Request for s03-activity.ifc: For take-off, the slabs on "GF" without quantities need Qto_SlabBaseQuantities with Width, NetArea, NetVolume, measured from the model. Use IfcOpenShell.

First a look at what the model holds.

```python
import ifcopenshell
import ifcopenshell.util.element
import ifcopenshell.util.unit

model = ifcopenshell.open("s03-activity.ifc")
print(model.schema)
for unit_type in ("LENGTHUNIT", "AREAUNIT", "VOLUMEUNIT"):
    print(unit_type, ifcopenshell.util.unit.calculate_unit_scale(model, unit_type))
storey = next(s for s in model.by_type("IfcBuildingStorey") if s.Name == "GF")
slabs = [e for e in ifcopenshell.util.element.get_decomposition(storey) if e.is_a("IfcSlab")]
for e in sorted(slabs, key=lambda e: e.id()):
    print(e.id(), e.is_a(), e.Name, list(ifcopenshell.util.element.get_psets(e, qtos_only=True)), sep=" | ")
```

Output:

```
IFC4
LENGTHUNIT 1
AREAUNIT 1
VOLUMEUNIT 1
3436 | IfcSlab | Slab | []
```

```python
import ifcopenshell
import ifcopenshell.api.pset
import ifcopenshell.geom
import ifcopenshell.util.element
import ifcopenshell.util.shape
import ifcopenshell.util.unit

model = ifcopenshell.open("s03-activity.ifc")
unit_scale = ifcopenshell.util.unit.calculate_unit_scale(model)
area_scale = ifcopenshell.util.unit.calculate_unit_scale(model, "AREAUNIT")
volume_scale = ifcopenshell.util.unit.calculate_unit_scale(model, "VOLUMEUNIT")
settings = ifcopenshell.geom.settings()

storey = next(s for s in model.by_type("IfcBuildingStorey") if s.Name == "GF")
slabs = [e for e in ifcopenshell.util.element.get_decomposition(storey) if e.is_a("IfcSlab")]

for e in sorted(slabs, key=lambda e: e.id()):
    if ifcopenshell.util.element.get_psets(e, qtos_only=True, should_inherit=False):
        continue
    # Geometry comes back in metres, in the element's own axes.
    shape = ifcopenshell.geom.create_shape(settings, e)
    values = {
        "Width": ifcopenshell.util.shape.get_z(shape.geometry) / unit_scale,
        "NetArea": ifcopenshell.util.shape.get_footprint_area(shape.geometry) / area_scale,
        "NetVolume": ifcopenshell.util.shape.get_volume(shape.geometry) / volume_scale,
    }
    qto = ifcopenshell.api.pset.add_qto(model, product=e, name="Qto_SlabBaseQuantities")
    ifcopenshell.api.pset.edit_qto(model, qto=qto, properties=values)
    print(e.id(), {k: round(v, 3) for k, v in values.items()})

model.write("s03-activity_rev.ifc")
```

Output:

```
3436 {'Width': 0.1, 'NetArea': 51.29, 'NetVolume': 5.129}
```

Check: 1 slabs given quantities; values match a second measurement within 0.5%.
